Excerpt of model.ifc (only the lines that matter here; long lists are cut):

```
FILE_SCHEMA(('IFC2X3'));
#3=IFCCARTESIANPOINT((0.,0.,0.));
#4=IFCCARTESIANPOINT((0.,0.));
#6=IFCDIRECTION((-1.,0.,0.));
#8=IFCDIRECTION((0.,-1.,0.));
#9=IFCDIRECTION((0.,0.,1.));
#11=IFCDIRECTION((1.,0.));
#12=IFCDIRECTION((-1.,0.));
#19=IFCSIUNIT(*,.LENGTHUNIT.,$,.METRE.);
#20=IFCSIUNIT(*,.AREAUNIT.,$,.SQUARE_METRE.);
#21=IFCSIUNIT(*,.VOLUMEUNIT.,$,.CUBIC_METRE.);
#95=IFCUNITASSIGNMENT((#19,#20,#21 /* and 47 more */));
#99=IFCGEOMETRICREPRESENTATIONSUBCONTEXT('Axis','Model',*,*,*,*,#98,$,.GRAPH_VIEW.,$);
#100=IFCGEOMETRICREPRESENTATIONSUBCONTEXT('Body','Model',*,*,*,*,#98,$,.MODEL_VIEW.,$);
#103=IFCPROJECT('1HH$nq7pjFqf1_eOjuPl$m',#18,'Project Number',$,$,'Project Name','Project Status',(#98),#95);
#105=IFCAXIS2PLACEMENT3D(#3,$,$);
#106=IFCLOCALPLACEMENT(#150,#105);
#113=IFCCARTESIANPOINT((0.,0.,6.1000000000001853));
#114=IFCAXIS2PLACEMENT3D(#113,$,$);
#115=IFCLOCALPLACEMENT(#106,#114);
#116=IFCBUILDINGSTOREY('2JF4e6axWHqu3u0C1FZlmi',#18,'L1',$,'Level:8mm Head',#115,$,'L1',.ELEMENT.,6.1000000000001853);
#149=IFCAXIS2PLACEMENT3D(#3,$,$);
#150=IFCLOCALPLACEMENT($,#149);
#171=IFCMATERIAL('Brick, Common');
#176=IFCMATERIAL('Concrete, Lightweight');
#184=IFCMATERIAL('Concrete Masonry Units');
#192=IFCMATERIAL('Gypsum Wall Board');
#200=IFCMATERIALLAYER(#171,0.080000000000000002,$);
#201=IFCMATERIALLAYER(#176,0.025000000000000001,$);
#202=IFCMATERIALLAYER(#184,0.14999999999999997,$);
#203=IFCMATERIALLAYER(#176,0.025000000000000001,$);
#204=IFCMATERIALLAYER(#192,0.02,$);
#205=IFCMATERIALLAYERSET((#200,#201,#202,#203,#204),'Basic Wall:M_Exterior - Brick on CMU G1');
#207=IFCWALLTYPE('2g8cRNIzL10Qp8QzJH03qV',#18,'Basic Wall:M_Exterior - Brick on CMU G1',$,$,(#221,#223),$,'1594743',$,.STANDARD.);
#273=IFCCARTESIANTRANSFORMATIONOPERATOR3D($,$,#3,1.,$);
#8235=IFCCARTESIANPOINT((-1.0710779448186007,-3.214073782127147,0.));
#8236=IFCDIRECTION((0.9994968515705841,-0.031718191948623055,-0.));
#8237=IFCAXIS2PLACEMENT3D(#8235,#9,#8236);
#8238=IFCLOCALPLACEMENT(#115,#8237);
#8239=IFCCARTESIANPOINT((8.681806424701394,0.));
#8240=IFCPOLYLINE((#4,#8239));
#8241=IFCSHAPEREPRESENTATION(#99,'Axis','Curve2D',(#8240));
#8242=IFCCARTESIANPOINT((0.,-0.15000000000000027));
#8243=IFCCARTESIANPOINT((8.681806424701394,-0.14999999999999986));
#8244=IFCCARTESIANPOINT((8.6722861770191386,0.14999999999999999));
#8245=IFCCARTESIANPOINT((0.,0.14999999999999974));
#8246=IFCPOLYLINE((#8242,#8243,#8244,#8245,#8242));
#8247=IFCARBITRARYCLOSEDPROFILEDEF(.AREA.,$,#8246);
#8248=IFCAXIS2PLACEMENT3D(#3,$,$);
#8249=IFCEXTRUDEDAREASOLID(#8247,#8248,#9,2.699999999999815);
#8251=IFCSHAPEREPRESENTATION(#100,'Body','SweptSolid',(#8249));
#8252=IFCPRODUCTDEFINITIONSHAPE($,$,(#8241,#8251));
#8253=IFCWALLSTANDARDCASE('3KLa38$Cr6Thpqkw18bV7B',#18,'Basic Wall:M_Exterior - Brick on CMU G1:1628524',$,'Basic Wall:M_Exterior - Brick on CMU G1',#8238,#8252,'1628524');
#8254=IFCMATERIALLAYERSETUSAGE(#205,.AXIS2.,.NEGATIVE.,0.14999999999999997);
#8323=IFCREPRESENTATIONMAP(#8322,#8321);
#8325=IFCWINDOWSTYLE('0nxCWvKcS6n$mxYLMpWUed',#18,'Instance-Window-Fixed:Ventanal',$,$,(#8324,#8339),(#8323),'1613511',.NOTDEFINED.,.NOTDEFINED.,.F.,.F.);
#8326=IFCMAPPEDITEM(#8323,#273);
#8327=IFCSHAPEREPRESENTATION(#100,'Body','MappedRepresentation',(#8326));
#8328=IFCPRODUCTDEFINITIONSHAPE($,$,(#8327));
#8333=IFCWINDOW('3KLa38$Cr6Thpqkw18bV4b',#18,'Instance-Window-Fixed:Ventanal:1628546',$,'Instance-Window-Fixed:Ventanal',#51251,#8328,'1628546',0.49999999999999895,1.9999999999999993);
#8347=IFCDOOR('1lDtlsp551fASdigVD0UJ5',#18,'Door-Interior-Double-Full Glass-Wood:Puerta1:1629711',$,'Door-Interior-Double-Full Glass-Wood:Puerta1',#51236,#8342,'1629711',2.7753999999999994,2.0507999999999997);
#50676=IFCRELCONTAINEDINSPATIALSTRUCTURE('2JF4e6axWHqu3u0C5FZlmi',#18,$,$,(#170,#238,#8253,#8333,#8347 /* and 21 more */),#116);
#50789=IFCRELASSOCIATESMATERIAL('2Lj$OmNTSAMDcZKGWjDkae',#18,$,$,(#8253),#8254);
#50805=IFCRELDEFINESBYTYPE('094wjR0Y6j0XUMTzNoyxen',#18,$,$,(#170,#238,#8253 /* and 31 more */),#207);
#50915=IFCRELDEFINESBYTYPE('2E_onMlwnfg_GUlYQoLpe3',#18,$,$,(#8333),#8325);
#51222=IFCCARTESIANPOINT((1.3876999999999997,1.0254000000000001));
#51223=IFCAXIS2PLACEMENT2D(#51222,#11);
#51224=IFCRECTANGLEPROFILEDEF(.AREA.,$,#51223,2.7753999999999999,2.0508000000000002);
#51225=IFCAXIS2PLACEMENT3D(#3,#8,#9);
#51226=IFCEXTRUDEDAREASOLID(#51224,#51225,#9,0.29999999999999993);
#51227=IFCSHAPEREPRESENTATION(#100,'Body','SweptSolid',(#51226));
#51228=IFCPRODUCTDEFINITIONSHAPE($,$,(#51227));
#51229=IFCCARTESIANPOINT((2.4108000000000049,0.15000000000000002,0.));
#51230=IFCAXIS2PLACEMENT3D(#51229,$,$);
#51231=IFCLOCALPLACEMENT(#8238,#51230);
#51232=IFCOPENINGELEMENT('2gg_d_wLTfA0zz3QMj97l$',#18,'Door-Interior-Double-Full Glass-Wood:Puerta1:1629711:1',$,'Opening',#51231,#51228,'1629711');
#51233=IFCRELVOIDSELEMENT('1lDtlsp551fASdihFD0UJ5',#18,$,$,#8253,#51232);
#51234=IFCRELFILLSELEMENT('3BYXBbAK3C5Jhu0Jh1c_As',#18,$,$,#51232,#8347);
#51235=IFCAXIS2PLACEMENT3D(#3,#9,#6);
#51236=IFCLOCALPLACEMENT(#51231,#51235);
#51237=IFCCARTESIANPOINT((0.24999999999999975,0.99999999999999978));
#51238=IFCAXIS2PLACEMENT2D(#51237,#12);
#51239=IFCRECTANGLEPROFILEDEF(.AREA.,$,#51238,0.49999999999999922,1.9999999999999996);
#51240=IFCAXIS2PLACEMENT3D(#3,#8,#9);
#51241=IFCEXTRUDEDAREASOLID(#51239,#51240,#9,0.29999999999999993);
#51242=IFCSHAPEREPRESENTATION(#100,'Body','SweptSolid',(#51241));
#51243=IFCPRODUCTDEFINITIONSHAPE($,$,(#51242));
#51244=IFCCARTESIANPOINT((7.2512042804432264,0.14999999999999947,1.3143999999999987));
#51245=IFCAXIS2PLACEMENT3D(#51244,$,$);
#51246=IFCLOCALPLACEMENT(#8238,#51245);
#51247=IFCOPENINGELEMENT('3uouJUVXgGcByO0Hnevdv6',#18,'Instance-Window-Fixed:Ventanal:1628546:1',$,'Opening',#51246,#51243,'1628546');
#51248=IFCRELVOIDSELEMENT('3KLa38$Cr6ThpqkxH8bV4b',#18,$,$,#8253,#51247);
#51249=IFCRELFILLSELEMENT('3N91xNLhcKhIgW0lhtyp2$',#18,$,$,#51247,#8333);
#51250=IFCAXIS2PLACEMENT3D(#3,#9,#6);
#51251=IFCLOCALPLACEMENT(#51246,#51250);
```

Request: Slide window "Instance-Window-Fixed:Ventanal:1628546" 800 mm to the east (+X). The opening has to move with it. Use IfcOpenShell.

```python
import ifcopenshell
import ifcopenshell.api.geometry
import ifcopenshell.util.placement

model = ifcopenshell.open("model.ifc")

window = model.by_guid("3KLa38$Cr6Thpqkw18bV4b")
opening = window.FillsVoids[0].RelatingOpeningElement
wall = opening.VoidsElements[0].RelatingBuildingElement

wall_matrix = ifcopenshell.util.placement.get_local_placement(wall.ObjectPlacement)
shift = wall_matrix[:3, 0] * 0.8
before = ifcopenshell.util.placement.get_local_placement(window.ObjectPlacement)[:3, 3].copy()

# The window is placed relative to its opening, so it follows when the opening moves.
matrix = ifcopenshell.util.placement.get_local_placement(opening.ObjectPlacement)
matrix[:3, 3] += shift
ifcopenshell.api.geometry.edit_object_placement(
    model, product=opening, matrix=matrix, is_si=False, should_transform_children=True
)

after = ifcopenshell.util.placement.get_local_placement(window.ObjectPlacement)[:3, 3]
print("window moved by", (after - before).round(3) + 0.0)

model.write("model_updated.ifc")
```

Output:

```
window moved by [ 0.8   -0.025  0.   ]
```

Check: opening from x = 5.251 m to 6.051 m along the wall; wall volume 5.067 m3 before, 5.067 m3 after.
